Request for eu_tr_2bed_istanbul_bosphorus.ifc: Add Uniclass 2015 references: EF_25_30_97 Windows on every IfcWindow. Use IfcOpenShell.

First a look at what the model holds.

```python
import ifcopenshell

model = ifcopenshell.open("eu_tr_2bed_istanbul_bosphorus.ifc")
print(model.schema)
print("classifications:", [c.Name for c in model.by_type("IfcClassification")])
for ifc_class in ("IfcDoor", "IfcRoof", "IfcStair", "IfcWall", "IfcWindow"):
    print(ifc_class, len(model.by_type(ifc_class)))
```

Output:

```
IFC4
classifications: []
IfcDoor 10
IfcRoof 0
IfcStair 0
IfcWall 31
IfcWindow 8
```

```python
import ifcopenshell
import ifcopenshell.api.classification

model = ifcopenshell.open("eu_tr_2bed_istanbul_bosphorus.ifc")

system = ifcopenshell.api.classification.add_classification(model, classification="Uniclass 2015")

codes = {
    "IfcWindow": ("EF_25_30_97", "Windows"),
}
for ifc_class, (code, name) in codes.items():
    products = model.by_type(ifc_class)
    ifcopenshell.api.classification.add_reference(
        model, products=products, classification=system, identification=code, name=name
    )
    print(code, len(products))

model.write("eu_tr_2bed_istanbul_bosphorus_rev.ifc")
```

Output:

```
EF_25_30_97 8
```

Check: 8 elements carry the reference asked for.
